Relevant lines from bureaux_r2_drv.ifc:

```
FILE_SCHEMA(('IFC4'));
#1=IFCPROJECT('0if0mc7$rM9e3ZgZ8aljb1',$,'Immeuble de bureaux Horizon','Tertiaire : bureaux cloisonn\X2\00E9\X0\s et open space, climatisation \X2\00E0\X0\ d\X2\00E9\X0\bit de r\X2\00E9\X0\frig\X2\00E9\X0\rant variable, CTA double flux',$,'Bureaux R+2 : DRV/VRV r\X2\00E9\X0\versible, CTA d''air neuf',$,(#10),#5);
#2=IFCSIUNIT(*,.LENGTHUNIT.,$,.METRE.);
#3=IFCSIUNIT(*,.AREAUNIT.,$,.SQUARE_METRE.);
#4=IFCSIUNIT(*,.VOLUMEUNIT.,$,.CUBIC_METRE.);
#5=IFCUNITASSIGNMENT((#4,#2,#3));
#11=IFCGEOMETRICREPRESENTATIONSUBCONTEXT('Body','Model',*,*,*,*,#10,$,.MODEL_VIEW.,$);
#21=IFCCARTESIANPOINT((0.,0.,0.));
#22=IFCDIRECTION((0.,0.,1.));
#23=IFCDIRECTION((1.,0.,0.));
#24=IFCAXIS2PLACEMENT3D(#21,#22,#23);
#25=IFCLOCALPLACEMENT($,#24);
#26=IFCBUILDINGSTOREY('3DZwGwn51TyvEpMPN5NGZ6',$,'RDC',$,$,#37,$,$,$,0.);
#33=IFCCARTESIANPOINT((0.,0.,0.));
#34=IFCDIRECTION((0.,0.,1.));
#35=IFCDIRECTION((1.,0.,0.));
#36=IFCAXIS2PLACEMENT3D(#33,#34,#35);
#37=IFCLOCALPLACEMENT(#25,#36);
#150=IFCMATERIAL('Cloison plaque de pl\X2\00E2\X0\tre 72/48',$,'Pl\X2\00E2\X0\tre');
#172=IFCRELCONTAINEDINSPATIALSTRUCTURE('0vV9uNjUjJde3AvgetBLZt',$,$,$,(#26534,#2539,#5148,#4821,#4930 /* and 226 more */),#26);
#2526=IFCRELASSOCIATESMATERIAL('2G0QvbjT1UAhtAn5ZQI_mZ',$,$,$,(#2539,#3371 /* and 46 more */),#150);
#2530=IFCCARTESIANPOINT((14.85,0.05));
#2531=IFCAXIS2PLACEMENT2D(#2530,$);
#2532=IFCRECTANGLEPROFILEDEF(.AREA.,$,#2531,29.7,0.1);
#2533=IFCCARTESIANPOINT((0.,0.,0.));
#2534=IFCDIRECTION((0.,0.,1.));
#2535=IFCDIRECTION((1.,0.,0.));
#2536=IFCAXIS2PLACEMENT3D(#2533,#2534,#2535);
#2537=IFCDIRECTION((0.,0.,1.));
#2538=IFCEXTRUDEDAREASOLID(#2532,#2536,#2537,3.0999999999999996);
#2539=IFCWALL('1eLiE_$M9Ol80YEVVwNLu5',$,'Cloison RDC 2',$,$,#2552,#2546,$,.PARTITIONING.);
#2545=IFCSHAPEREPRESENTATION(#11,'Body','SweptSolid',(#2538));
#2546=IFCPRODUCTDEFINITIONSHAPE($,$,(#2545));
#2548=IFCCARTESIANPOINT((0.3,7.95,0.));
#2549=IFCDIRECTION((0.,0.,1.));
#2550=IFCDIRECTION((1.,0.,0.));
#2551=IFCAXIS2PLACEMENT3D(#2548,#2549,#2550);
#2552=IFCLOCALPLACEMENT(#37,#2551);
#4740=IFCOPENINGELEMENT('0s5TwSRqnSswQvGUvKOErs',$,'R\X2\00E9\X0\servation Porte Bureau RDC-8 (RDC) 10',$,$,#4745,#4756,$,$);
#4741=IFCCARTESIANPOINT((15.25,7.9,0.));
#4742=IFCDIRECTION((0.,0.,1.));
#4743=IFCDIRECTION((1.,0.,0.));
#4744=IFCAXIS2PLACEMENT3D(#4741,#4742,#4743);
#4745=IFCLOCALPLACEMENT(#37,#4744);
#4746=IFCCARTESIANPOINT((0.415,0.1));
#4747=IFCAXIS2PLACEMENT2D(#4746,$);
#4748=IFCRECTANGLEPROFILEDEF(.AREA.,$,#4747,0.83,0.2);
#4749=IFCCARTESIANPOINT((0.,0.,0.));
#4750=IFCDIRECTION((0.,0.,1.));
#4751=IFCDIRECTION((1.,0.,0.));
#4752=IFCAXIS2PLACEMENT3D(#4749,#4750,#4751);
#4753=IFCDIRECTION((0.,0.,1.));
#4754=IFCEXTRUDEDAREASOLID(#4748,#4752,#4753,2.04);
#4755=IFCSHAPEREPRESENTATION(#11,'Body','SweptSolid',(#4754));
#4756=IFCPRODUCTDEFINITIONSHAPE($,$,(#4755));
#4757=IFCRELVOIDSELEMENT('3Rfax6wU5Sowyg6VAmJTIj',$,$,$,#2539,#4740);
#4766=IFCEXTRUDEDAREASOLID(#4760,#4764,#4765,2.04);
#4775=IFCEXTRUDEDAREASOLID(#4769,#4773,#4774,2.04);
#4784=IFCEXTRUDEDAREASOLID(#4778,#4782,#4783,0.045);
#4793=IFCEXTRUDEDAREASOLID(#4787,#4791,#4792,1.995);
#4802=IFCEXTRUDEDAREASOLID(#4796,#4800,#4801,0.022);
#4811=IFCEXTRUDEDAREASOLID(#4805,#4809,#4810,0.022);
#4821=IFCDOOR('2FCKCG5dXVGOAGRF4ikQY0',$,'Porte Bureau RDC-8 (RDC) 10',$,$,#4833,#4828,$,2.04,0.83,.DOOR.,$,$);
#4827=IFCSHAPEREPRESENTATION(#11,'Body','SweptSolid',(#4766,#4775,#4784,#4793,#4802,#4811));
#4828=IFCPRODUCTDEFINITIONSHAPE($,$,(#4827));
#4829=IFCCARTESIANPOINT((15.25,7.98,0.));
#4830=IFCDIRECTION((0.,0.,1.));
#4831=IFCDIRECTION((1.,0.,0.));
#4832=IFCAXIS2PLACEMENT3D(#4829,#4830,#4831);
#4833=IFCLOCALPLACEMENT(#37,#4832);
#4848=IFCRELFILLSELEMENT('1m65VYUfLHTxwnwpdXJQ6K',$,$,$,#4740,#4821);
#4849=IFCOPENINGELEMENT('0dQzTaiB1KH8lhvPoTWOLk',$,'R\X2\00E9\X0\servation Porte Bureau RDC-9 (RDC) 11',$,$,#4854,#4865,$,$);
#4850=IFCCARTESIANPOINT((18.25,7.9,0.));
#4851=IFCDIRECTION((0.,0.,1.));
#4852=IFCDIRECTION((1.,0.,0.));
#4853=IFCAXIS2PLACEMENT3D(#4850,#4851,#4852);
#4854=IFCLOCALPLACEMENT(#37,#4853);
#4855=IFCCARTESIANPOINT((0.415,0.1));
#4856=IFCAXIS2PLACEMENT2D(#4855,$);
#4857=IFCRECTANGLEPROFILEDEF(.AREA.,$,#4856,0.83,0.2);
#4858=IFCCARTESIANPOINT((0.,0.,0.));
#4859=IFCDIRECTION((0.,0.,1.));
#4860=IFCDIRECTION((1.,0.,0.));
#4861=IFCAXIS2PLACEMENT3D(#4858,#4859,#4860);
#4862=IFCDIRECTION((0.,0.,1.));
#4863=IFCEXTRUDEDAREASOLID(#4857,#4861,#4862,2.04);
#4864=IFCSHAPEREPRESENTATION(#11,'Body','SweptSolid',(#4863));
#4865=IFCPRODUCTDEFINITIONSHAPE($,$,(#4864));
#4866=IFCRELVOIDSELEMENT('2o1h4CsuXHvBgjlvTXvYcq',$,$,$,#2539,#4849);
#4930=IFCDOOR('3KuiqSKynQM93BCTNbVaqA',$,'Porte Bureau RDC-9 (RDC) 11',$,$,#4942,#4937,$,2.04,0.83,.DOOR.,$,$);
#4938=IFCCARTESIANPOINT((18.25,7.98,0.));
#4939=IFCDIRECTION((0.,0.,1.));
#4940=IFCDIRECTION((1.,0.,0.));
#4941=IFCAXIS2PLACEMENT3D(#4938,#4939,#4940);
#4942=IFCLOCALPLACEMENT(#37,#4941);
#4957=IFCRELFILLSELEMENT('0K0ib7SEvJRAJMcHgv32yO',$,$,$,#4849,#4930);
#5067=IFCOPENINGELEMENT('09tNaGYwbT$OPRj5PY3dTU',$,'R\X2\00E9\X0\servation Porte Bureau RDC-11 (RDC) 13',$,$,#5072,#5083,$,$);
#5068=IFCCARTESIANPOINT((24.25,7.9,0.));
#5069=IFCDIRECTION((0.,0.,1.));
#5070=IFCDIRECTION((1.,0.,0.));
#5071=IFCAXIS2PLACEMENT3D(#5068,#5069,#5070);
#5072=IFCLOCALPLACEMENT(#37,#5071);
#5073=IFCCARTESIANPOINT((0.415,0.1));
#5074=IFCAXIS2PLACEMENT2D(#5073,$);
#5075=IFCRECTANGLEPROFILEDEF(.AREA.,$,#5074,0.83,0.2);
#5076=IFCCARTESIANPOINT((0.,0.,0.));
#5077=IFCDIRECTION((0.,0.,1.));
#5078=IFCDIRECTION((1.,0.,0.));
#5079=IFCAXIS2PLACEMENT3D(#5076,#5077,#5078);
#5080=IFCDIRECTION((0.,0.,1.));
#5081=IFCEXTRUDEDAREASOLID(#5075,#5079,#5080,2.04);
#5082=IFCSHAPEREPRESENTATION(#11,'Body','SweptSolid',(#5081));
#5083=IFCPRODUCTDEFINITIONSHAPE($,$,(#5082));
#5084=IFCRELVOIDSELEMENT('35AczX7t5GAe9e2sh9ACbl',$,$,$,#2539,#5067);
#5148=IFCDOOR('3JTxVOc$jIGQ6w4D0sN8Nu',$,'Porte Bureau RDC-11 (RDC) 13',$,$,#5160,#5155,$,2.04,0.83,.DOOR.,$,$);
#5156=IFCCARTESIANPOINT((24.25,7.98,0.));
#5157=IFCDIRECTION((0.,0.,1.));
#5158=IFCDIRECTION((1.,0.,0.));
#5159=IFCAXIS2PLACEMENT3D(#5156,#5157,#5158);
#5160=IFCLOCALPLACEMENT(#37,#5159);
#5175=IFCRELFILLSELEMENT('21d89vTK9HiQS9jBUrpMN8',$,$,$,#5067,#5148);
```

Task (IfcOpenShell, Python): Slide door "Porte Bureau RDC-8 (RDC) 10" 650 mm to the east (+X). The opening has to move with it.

```python
import ifcopenshell
import ifcopenshell.api.geometry
import ifcopenshell.util.placement

model = ifcopenshell.open("bureaux_r2_drv.ifc")

door = model.by_guid("2FCKCG5dXVGOAGRF4ikQY0")
opening = door.FillsVoids[0].RelatingOpeningElement
wall = opening.VoidsElements[0].RelatingBuildingElement

wall_matrix = ifcopenshell.util.placement.get_local_placement(wall.ObjectPlacement)
shift = wall_matrix[:3, 0] * 0.65
before = ifcopenshell.util.placement.get_local_placement(door.ObjectPlacement)[:3, 3].copy()

# The door is not placed relative to its opening, so move both.
for product in (opening, door):
    matrix = ifcopenshell.util.placement.get_local_placement(product.ObjectPlacement)
    matrix[:3, 3] += shift
    ifcopenshell.api.geometry.edit_object_placement(model, product=product, matrix=matrix, is_si=False)

after = ifcopenshell.util.placement.get_local_placement(door.ObjectPlacement)[:3, 3]
print("door moved by", (after - before).round(3) + 0.0)

model.write("bureaux_r2_drv_updated.ifc")
```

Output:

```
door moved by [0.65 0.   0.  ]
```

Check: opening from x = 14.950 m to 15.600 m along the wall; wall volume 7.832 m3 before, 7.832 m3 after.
